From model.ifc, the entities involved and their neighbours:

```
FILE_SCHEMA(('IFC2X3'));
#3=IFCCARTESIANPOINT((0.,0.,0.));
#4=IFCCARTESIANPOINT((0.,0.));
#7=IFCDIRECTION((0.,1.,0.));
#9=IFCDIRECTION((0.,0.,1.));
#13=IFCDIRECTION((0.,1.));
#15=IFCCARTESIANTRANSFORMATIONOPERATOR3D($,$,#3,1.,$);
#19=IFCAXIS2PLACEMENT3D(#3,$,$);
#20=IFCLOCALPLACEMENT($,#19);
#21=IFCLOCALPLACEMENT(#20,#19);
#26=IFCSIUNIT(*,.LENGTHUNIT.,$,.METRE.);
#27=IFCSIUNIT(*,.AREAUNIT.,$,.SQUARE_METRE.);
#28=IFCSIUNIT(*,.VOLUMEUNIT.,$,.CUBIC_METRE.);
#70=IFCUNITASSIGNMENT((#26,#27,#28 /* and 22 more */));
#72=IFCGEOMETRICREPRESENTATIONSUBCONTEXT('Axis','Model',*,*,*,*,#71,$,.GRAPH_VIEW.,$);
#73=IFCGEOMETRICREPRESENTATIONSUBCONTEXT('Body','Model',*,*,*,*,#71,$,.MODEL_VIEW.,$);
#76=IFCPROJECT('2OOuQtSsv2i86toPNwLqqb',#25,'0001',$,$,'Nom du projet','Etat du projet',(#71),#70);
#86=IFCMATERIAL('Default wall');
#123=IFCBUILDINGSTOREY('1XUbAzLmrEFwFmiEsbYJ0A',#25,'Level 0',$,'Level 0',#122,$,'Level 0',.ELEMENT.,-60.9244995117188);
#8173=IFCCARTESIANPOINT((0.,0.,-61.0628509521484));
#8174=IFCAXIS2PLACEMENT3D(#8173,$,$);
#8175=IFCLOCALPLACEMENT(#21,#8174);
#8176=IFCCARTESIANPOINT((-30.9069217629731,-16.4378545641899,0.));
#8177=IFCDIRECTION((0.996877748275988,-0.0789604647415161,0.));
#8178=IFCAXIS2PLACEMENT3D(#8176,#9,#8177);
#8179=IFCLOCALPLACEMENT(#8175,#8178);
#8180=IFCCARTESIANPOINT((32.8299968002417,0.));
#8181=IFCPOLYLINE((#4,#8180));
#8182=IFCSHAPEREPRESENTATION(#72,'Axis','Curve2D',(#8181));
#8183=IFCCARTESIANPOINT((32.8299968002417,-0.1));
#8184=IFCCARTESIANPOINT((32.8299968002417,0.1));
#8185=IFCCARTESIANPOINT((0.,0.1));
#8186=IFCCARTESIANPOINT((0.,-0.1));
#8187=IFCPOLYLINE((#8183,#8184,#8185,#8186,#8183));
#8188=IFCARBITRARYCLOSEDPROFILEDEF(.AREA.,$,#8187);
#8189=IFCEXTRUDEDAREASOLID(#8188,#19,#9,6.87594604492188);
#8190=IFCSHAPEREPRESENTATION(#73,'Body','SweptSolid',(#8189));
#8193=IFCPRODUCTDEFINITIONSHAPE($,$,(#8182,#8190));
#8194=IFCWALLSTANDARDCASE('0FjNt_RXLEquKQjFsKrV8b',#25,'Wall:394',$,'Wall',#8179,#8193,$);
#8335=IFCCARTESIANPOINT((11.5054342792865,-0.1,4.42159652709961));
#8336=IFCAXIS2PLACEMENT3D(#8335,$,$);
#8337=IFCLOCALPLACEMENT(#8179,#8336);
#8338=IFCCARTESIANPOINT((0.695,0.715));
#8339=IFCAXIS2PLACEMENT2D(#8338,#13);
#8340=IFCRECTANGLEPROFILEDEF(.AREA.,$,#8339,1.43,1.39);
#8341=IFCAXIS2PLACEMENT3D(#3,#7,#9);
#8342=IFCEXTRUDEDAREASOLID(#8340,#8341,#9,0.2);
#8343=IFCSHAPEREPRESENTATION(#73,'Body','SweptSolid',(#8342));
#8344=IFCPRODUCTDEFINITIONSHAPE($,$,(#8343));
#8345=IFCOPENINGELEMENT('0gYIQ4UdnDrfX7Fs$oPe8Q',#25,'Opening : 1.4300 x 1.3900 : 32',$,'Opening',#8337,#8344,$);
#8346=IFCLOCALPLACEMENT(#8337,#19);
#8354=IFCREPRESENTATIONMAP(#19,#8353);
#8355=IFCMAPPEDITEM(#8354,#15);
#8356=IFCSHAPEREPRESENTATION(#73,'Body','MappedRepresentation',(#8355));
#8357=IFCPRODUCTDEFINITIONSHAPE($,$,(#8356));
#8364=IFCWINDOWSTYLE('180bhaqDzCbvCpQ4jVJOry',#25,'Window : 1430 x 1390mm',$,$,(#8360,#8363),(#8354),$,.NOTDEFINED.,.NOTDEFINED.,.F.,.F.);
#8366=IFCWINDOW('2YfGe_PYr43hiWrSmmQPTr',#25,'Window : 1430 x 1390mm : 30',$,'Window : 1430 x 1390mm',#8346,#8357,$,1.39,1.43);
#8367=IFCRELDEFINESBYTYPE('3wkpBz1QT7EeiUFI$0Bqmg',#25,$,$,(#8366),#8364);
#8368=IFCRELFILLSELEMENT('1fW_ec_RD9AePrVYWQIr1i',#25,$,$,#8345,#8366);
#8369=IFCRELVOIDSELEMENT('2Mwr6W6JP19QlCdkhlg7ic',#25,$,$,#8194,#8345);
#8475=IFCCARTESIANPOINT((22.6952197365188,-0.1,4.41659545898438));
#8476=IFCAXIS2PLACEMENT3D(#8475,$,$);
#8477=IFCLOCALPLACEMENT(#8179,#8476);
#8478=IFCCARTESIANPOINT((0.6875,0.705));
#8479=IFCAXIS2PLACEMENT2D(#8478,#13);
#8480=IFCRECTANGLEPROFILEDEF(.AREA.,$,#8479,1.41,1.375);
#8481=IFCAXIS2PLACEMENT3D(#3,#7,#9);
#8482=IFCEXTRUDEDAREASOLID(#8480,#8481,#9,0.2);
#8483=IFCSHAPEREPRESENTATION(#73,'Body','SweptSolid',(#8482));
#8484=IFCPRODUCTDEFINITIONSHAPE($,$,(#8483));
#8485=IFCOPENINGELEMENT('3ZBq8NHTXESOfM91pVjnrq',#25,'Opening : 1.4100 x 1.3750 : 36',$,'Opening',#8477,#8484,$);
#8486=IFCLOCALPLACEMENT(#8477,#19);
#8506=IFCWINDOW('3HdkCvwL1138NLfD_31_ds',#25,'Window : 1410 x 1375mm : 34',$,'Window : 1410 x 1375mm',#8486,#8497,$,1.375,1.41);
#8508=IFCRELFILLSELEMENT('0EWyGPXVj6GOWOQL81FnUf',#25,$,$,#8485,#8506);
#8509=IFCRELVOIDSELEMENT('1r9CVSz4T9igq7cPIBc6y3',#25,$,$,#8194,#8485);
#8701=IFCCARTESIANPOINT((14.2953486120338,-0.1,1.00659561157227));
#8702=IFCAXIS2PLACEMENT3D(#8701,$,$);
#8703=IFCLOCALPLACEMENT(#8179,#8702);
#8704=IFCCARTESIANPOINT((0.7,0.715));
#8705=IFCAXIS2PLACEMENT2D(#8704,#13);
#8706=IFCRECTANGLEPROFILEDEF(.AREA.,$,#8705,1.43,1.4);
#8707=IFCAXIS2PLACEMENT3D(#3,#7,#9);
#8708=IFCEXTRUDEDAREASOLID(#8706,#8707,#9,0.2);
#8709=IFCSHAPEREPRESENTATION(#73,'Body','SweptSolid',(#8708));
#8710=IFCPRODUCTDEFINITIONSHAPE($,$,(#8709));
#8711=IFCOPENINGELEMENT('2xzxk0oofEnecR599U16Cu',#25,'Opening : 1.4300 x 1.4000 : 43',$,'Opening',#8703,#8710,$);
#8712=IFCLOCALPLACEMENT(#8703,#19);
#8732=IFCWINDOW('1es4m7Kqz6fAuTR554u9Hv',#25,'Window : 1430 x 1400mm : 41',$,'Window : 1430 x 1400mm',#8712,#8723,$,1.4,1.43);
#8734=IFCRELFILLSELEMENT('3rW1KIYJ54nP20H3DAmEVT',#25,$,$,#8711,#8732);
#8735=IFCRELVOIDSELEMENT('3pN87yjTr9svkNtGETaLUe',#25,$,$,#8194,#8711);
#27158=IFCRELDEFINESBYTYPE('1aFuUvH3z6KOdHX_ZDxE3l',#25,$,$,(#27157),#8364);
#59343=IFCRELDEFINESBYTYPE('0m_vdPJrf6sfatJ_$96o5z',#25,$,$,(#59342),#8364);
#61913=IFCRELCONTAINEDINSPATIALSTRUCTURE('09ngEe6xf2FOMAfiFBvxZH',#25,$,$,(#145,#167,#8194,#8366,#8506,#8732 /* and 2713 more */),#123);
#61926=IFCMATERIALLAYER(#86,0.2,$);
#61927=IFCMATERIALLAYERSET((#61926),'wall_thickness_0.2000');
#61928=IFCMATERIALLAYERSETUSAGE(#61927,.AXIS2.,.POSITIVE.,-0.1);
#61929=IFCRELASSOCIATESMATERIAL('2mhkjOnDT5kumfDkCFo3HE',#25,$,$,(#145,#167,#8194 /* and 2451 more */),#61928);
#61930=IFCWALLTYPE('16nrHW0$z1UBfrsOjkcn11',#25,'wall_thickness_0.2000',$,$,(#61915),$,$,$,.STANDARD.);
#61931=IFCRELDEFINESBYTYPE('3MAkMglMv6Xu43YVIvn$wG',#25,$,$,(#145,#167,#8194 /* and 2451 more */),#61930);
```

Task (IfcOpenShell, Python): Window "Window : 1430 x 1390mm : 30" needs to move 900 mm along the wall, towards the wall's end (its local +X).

```python
import ifcopenshell
import ifcopenshell.api.geometry
import ifcopenshell.util.placement

model = ifcopenshell.open("model.ifc")

window = model.by_guid("2YfGe_PYr43hiWrSmmQPTr")
opening = window.FillsVoids[0].RelatingOpeningElement
wall = opening.VoidsElements[0].RelatingBuildingElement

wall_matrix = ifcopenshell.util.placement.get_local_placement(wall.ObjectPlacement)
shift = wall_matrix[:3, 0] * 0.9
before = ifcopenshell.util.placement.get_local_placement(window.ObjectPlacement)[:3, 3].copy()

# The window is placed relative to its opening, so it follows when the opening moves.
matrix = ifcopenshell.util.placement.get_local_placement(opening.ObjectPlacement)
matrix[:3, 3] += shift
ifcopenshell.api.geometry.edit_object_placement(
    model, product=opening, matrix=matrix, is_si=False, should_transform_children=True
)

after = ifcopenshell.util.placement.get_local_placement(window.ObjectPlacement)[:3, 3]
print("window moved by", (after - before).round(3) + 0.0)

model.write("model-out.ifc")
```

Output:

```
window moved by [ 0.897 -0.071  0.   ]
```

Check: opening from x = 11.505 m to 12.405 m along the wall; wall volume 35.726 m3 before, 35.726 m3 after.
